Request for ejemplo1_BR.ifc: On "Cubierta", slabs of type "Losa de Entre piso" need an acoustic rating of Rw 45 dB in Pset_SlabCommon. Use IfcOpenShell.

First a look at what the model holds.

```python
import ifcopenshell
import ifcopenshell.util.element

model = ifcopenshell.open("ejemplo1_BR.ifc")
print(model.schema)
storey = next(s for s in model.by_type("IfcBuildingStorey") if s.Name == "Cubierta")
slabs = [e for e in ifcopenshell.util.element.get_decomposition(storey) if e.is_a("IfcSlab")]
seen = {}
for e in slabs:
    element_type = ifcopenshell.util.element.get_type(e)
    key = (element_type.Name if element_type != e and element_type else None, ifcopenshell.util.element.get_pset(e, "Pset_SlabCommon", "AcousticRating"))
    seen[key] = seen.get(key, 0) + 1
for (name, value), count in sorted(seen.items(), key=str):
    print(count, "x", name, "|", value)
```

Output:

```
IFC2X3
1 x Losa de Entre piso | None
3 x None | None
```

```python
import ifcopenshell
import ifcopenshell.api.pset
import ifcopenshell.util.element

model = ifcopenshell.open("ejemplo1_BR.ifc")

storey = next(s for s in model.by_type("IfcBuildingStorey") if s.Name == "Cubierta")
slabs = [e for e in ifcopenshell.util.element.get_decomposition(storey) if e.is_a("IfcSlab")]

count = 0
for e in slabs:
    element_type = ifcopenshell.util.element.get_type(e)
    if element_type in (None, e) or element_type.Name != "Losa de Entre piso":
        continue
    # add_pset returns the element's existing set when there is one.
    pset = ifcopenshell.api.pset.add_pset(model, product=e, name="Pset_SlabCommon")
    ifcopenshell.api.pset.edit_pset(model, pset=pset, properties={"AcousticRating": "Rw 45 dB"})
    count += 1

print(count, "slabs updated")

model.write("ejemplo1_BR_rev.ifc")
```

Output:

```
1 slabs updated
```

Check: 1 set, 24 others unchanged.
